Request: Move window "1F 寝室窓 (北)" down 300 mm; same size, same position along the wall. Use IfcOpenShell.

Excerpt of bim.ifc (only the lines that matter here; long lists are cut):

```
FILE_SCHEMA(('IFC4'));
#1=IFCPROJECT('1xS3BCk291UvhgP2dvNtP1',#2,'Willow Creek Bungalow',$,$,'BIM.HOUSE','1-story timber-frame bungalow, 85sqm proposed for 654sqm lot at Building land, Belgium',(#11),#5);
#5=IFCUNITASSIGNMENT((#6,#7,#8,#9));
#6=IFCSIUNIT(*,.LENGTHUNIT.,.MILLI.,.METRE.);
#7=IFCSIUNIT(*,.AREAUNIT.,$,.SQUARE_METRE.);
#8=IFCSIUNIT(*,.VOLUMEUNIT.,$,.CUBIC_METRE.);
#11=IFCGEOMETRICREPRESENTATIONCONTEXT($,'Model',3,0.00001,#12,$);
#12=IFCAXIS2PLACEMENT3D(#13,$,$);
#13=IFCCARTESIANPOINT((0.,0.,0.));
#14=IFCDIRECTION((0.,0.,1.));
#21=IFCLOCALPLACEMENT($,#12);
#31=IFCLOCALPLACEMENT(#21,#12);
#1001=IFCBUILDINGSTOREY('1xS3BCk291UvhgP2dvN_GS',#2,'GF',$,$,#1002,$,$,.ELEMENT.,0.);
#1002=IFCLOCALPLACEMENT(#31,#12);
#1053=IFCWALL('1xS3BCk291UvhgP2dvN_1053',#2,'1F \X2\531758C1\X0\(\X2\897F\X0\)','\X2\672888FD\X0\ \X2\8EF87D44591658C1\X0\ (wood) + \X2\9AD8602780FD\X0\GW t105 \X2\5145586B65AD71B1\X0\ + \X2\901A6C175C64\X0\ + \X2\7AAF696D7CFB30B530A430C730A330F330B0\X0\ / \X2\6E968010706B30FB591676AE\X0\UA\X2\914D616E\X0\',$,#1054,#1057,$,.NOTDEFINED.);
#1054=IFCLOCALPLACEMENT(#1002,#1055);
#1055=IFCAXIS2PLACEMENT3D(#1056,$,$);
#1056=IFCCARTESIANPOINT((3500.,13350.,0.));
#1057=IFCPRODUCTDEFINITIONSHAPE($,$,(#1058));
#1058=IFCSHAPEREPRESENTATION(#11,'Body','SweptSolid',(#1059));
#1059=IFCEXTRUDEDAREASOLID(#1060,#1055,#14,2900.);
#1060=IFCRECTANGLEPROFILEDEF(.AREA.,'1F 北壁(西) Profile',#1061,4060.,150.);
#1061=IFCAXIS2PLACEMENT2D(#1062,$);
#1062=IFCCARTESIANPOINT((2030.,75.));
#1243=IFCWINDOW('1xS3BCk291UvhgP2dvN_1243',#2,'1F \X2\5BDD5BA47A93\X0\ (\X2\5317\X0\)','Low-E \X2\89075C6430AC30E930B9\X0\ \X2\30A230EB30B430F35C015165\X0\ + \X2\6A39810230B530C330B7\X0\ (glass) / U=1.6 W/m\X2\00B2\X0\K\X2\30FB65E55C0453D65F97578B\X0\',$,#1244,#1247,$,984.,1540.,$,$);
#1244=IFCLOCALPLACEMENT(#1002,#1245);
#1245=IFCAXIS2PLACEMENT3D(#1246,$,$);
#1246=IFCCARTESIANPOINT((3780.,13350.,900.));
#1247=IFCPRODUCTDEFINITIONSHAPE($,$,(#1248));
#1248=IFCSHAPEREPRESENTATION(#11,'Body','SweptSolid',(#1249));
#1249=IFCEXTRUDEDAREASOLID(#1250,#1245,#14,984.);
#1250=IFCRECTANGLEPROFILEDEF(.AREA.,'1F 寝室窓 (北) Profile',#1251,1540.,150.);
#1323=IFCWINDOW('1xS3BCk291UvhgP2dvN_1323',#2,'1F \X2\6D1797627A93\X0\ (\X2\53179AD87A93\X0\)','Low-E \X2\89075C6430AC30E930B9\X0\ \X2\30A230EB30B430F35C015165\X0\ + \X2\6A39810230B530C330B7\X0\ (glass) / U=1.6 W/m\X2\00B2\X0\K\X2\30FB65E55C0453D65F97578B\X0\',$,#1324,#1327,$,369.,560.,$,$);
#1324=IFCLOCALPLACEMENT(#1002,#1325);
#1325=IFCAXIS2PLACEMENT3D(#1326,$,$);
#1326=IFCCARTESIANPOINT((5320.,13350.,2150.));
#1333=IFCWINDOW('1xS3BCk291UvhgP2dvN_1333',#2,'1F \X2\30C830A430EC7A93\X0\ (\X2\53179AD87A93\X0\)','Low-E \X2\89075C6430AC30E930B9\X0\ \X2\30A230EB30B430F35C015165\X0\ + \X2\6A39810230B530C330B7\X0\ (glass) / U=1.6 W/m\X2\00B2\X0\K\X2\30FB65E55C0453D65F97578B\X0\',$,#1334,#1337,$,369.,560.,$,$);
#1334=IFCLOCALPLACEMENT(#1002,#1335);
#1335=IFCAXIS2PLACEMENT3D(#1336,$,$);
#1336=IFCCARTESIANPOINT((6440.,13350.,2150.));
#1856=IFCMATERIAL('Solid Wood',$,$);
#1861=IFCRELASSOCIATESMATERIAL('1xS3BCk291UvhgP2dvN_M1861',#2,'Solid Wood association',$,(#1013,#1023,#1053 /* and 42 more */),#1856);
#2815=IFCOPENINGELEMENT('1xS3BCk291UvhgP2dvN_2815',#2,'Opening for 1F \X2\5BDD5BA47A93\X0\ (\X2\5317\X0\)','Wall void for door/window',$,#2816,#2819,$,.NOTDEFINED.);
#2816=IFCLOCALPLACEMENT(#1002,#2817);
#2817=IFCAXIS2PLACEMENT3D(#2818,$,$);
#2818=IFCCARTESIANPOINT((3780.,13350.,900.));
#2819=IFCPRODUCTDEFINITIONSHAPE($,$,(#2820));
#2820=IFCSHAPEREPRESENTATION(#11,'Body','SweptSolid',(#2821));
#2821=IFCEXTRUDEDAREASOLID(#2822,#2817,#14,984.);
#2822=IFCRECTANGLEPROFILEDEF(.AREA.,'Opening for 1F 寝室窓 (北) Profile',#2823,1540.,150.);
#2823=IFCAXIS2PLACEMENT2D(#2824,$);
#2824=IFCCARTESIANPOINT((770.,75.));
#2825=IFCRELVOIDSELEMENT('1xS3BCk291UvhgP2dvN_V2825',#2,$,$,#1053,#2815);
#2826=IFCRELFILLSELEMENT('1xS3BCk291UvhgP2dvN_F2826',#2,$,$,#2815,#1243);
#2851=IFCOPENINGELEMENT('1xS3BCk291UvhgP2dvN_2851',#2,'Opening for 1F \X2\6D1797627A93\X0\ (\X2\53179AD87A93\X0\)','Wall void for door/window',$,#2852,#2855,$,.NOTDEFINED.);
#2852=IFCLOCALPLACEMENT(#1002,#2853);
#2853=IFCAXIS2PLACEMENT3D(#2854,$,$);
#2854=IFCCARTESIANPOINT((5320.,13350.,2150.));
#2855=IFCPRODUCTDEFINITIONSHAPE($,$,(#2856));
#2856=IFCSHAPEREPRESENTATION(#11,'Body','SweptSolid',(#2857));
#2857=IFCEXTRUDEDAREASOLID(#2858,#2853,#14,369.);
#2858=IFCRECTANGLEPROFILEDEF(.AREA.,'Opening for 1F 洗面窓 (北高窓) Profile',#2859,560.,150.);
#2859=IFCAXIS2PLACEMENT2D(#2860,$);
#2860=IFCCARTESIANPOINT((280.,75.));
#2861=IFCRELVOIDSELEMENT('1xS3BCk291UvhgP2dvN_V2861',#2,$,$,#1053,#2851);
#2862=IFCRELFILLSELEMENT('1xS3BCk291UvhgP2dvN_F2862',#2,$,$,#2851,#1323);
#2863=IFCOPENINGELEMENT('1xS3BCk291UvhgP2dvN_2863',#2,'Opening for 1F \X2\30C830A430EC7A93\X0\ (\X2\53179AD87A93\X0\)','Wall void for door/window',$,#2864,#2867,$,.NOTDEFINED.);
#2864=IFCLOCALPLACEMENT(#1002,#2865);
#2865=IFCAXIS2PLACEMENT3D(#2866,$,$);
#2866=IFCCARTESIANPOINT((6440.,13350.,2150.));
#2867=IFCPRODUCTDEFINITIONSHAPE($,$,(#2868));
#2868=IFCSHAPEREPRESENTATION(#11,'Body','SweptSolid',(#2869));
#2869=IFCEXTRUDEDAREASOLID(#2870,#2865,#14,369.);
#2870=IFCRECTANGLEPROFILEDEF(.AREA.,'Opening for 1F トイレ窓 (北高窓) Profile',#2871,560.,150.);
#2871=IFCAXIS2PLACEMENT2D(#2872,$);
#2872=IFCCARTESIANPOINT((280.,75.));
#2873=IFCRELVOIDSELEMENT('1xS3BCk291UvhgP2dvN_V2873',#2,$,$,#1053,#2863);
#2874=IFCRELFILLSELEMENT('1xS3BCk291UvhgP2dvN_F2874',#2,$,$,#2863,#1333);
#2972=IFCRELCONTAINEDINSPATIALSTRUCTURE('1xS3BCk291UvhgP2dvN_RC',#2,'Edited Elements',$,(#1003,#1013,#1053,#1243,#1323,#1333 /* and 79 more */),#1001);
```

```python
import numpy as np
import ifcopenshell
import ifcopenshell.api.geometry
import ifcopenshell.util.placement
import ifcopenshell.util.unit

model = ifcopenshell.open("bim.ifc")
unit_scale = ifcopenshell.util.unit.calculate_unit_scale(model)

window = model.by_guid("1xS3BCk291UvhgP2dvN_1243")
opening = window.FillsVoids[0].RelatingOpeningElement
dz = -0.3 / unit_scale

shift = np.array([0.0, 0.0, dz])
# The window is not placed relative to its opening, so move both.
for product in (opening, window):
    matrix = ifcopenshell.util.placement.get_local_placement(product.ObjectPlacement)
    matrix[:3, 3] += shift
    ifcopenshell.api.geometry.edit_object_placement(model, product=product, matrix=matrix, is_si=False)

print(f"moved by {dz * unit_scale:+.3f} m")

model.write("bim_updated.ifc")
```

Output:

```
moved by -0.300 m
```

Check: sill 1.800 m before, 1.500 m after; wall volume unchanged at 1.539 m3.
